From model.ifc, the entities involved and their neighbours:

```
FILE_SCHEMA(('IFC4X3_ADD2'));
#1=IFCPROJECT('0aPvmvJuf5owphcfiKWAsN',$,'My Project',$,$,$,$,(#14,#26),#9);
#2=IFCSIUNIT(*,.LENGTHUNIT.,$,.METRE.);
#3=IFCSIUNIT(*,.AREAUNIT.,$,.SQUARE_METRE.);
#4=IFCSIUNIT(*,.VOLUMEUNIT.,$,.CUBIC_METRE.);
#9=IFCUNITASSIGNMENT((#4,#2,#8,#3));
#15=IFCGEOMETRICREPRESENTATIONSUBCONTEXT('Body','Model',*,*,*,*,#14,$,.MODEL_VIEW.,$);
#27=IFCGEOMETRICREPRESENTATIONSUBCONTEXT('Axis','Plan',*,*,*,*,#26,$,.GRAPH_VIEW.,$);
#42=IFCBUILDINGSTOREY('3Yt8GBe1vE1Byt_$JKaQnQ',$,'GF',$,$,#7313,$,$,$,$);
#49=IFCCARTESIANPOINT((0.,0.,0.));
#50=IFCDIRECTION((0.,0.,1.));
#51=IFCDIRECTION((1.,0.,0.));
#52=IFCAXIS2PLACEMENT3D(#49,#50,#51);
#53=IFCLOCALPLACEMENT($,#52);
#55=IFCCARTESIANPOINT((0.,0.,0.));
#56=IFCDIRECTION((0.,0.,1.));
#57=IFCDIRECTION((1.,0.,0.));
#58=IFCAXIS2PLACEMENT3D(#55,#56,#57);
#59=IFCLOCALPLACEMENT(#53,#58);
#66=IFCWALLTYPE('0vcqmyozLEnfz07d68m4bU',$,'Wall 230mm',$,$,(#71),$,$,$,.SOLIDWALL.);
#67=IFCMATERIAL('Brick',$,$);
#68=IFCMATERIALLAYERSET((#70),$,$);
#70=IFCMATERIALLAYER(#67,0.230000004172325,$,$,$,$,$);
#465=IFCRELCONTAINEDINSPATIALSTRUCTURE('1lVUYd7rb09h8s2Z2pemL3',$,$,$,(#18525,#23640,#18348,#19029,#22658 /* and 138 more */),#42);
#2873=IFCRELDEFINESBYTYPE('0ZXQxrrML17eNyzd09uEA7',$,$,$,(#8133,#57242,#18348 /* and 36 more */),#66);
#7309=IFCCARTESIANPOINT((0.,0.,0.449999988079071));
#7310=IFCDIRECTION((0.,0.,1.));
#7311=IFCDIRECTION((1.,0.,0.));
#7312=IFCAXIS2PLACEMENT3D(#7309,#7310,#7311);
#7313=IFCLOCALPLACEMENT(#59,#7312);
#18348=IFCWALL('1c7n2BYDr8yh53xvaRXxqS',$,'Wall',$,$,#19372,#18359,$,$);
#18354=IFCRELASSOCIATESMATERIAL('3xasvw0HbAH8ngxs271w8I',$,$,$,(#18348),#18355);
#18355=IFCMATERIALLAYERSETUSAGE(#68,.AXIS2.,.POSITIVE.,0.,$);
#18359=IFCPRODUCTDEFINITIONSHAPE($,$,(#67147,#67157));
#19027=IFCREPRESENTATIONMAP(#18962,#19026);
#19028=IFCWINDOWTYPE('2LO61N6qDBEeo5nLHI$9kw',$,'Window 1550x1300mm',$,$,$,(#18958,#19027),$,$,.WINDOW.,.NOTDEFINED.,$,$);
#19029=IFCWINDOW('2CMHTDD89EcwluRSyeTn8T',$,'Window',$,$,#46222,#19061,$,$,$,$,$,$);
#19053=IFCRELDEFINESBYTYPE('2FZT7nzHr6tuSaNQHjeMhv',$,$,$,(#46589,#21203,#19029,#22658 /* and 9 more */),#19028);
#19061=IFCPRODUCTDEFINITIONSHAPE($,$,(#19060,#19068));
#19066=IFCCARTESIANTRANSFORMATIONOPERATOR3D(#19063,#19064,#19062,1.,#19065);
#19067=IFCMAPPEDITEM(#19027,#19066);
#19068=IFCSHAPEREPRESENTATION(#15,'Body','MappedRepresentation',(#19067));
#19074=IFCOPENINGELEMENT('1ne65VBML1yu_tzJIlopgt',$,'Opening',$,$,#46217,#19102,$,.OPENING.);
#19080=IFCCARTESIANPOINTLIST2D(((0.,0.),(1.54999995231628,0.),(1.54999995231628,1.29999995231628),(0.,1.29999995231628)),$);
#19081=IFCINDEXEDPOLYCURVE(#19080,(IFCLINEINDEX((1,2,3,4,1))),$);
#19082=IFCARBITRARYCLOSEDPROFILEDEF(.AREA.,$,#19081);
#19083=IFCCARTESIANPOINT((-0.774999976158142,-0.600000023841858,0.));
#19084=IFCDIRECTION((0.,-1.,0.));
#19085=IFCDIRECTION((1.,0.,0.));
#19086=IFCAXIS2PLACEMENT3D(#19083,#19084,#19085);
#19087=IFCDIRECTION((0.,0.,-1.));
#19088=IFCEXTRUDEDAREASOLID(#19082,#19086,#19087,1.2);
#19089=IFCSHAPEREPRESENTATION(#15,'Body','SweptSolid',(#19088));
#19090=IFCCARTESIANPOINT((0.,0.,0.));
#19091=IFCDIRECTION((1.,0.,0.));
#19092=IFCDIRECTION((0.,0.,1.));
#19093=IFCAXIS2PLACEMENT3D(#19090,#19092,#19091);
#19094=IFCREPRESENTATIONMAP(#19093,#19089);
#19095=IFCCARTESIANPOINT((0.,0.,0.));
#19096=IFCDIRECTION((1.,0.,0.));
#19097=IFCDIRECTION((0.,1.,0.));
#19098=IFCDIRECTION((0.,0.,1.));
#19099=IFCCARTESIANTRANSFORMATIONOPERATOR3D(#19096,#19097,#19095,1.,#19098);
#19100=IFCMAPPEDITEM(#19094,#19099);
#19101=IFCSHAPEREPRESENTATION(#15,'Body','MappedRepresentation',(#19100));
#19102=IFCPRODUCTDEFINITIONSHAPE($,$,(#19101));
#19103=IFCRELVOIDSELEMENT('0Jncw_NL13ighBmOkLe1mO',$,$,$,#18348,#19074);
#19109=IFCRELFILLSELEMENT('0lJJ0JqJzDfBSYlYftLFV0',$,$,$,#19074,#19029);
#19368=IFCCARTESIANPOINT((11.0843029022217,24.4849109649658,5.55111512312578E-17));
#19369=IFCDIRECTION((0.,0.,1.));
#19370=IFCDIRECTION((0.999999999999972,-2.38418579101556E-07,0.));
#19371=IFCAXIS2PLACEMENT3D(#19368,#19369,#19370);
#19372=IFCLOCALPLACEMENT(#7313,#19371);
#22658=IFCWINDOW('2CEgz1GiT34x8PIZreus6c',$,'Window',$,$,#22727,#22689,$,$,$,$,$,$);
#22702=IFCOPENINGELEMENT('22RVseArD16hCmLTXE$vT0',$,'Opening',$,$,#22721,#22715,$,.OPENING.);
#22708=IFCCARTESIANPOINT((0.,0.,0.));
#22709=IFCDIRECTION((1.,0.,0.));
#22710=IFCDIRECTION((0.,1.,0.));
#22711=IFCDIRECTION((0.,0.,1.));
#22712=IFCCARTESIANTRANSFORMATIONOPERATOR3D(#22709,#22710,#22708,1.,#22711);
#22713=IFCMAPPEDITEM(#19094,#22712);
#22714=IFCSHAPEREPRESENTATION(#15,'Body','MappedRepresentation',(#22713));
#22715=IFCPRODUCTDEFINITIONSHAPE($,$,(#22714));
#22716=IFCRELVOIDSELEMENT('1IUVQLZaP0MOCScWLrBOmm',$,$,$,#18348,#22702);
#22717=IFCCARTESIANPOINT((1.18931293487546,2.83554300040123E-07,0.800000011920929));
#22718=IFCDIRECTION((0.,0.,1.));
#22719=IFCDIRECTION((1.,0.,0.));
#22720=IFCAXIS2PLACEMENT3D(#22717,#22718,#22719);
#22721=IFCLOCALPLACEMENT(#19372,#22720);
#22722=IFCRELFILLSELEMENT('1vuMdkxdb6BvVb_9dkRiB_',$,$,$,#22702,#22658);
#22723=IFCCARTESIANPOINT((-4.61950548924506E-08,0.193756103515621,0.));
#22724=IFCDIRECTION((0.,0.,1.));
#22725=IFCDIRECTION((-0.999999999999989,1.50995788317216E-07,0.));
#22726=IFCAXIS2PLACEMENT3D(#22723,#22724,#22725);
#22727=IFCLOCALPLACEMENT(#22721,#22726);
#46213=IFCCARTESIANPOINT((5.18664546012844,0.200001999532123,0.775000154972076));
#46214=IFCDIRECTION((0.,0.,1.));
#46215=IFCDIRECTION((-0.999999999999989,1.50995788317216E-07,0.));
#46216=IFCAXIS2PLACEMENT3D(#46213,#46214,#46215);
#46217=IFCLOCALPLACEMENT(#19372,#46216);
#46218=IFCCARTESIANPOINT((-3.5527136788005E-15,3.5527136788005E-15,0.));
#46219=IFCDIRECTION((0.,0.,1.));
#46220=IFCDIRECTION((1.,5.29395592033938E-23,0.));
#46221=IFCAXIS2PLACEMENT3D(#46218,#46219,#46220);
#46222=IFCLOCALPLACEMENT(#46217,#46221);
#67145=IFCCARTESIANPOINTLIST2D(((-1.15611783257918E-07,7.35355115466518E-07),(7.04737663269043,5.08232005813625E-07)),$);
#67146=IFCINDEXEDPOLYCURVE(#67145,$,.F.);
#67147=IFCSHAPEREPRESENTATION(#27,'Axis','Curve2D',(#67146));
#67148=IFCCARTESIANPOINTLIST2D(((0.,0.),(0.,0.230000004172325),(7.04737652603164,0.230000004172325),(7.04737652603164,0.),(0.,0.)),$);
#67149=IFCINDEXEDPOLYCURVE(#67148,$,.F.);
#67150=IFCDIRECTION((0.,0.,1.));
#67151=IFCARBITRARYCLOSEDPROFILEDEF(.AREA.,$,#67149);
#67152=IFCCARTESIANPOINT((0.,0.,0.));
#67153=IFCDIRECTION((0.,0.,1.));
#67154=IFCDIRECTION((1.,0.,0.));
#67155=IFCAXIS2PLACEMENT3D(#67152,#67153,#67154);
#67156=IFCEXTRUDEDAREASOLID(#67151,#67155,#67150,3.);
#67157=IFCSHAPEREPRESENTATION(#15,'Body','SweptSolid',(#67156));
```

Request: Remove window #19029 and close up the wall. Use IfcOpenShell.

```python
import ifcopenshell
import ifcopenshell.api.feature
import ifcopenshell.api.root
import ifcopenshell.geom
import ifcopenshell.util.shape

model = ifcopenshell.open("model.ifc")
settings = ifcopenshell.geom.settings()


def volume(element):
    """Net volume in cubic metres, openings subtracted."""
    shape = ifcopenshell.geom.create_shape(settings, element)
    return ifcopenshell.util.shape.get_volume(shape.geometry)


window = model.by_id(19029)
opening = window.FillsVoids[0].RelatingOpeningElement
wall = opening.VoidsElements[0].RelatingBuildingElement
before = volume(wall)

ifcopenshell.api.root.remove_product(model, product=window)
ifcopenshell.api.feature.remove_feature(model, feature=opening)

after = volume(wall)

print(f"wall volume {before:.3f} -> {after:.3f} m3")

model.write("model_rev.ifc")
```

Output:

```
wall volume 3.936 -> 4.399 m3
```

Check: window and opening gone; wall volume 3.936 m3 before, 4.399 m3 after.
